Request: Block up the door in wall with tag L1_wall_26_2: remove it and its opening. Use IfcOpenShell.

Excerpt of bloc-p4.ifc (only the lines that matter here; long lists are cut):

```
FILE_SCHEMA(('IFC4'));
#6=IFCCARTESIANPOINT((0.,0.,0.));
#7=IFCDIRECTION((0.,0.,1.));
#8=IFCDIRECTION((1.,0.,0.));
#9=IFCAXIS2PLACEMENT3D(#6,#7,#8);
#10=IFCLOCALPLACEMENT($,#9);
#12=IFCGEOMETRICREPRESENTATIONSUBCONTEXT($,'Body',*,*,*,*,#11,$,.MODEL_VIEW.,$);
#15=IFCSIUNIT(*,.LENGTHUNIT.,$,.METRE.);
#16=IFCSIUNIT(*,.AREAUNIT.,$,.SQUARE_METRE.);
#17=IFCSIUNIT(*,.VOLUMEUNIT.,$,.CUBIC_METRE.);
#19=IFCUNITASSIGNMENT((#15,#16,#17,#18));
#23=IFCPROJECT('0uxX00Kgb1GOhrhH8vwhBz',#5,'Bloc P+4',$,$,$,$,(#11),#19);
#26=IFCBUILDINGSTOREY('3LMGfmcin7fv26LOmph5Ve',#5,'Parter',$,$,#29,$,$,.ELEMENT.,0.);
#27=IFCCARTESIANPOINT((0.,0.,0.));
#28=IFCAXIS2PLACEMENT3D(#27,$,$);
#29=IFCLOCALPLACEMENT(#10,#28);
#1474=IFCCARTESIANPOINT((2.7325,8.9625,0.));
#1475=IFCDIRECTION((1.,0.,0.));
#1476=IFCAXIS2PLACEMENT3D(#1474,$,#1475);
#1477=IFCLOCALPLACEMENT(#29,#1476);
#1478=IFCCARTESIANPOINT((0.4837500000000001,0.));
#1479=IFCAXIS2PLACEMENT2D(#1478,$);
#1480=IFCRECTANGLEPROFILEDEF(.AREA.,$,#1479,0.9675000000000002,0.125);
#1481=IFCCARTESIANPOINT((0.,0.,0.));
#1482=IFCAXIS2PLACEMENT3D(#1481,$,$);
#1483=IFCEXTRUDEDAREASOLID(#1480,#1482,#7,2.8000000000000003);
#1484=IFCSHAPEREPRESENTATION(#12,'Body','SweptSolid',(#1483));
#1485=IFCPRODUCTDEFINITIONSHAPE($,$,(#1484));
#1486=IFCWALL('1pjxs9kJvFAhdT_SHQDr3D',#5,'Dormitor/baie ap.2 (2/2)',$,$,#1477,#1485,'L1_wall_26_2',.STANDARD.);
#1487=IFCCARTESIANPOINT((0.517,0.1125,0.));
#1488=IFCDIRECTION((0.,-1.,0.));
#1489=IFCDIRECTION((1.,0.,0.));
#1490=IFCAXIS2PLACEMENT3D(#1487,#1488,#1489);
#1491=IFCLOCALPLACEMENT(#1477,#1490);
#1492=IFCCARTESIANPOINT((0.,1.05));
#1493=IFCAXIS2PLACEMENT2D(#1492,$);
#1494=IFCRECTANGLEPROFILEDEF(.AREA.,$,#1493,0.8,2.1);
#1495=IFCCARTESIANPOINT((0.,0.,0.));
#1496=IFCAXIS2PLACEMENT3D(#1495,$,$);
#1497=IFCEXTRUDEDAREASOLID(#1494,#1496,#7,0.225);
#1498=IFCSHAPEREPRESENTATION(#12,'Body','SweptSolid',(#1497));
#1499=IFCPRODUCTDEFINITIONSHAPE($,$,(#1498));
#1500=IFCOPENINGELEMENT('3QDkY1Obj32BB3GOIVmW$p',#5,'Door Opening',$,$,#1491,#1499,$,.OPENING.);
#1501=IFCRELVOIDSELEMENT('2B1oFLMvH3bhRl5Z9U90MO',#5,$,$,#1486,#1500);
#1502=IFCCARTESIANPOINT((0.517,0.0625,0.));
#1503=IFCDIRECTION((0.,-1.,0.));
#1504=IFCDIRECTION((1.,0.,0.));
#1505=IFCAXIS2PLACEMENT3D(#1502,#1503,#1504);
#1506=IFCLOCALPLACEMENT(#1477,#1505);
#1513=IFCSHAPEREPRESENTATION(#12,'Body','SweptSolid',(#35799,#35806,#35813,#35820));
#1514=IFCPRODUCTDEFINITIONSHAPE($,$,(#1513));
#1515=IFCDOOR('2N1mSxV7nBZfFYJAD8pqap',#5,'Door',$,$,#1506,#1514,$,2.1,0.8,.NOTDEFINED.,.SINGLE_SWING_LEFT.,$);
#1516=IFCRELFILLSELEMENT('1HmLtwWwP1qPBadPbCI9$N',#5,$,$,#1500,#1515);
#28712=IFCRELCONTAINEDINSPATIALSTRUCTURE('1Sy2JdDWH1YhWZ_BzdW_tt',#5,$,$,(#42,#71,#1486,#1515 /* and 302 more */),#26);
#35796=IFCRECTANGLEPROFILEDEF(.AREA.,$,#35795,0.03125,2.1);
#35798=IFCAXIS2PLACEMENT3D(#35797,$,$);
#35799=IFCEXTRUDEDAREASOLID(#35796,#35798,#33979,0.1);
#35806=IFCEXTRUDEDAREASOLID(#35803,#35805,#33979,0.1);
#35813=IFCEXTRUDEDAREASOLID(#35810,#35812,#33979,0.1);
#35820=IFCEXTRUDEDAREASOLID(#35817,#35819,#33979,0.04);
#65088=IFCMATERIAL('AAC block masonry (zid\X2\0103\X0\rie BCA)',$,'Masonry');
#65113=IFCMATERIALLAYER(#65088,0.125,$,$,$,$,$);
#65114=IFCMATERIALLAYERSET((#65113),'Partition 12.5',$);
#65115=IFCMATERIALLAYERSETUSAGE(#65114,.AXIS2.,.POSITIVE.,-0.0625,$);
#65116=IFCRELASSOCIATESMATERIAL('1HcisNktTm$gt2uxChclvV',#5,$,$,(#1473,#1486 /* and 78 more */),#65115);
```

```python
import ifcopenshell
import ifcopenshell.api.feature
import ifcopenshell.api.root
import ifcopenshell.geom
import ifcopenshell.util.shape

model = ifcopenshell.open("bloc-p4.ifc")
settings = ifcopenshell.geom.settings()


def volume(element):
    """Net volume in cubic metres, openings subtracted."""
    shape = ifcopenshell.geom.create_shape(settings, element)
    return ifcopenshell.util.shape.get_volume(shape.geometry)


door = model.by_id(1515)
opening = door.FillsVoids[0].RelatingOpeningElement
wall = opening.VoidsElements[0].RelatingBuildingElement
before = volume(wall)

ifcopenshell.api.root.remove_product(model, product=door)
ifcopenshell.api.feature.remove_feature(model, feature=opening)

after = volume(wall)

print(f"wall volume {before:.3f} -> {after:.3f} m3")

model.write("bloc-p4-out.ifc")
```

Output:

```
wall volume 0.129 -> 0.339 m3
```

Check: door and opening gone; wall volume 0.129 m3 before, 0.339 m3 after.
